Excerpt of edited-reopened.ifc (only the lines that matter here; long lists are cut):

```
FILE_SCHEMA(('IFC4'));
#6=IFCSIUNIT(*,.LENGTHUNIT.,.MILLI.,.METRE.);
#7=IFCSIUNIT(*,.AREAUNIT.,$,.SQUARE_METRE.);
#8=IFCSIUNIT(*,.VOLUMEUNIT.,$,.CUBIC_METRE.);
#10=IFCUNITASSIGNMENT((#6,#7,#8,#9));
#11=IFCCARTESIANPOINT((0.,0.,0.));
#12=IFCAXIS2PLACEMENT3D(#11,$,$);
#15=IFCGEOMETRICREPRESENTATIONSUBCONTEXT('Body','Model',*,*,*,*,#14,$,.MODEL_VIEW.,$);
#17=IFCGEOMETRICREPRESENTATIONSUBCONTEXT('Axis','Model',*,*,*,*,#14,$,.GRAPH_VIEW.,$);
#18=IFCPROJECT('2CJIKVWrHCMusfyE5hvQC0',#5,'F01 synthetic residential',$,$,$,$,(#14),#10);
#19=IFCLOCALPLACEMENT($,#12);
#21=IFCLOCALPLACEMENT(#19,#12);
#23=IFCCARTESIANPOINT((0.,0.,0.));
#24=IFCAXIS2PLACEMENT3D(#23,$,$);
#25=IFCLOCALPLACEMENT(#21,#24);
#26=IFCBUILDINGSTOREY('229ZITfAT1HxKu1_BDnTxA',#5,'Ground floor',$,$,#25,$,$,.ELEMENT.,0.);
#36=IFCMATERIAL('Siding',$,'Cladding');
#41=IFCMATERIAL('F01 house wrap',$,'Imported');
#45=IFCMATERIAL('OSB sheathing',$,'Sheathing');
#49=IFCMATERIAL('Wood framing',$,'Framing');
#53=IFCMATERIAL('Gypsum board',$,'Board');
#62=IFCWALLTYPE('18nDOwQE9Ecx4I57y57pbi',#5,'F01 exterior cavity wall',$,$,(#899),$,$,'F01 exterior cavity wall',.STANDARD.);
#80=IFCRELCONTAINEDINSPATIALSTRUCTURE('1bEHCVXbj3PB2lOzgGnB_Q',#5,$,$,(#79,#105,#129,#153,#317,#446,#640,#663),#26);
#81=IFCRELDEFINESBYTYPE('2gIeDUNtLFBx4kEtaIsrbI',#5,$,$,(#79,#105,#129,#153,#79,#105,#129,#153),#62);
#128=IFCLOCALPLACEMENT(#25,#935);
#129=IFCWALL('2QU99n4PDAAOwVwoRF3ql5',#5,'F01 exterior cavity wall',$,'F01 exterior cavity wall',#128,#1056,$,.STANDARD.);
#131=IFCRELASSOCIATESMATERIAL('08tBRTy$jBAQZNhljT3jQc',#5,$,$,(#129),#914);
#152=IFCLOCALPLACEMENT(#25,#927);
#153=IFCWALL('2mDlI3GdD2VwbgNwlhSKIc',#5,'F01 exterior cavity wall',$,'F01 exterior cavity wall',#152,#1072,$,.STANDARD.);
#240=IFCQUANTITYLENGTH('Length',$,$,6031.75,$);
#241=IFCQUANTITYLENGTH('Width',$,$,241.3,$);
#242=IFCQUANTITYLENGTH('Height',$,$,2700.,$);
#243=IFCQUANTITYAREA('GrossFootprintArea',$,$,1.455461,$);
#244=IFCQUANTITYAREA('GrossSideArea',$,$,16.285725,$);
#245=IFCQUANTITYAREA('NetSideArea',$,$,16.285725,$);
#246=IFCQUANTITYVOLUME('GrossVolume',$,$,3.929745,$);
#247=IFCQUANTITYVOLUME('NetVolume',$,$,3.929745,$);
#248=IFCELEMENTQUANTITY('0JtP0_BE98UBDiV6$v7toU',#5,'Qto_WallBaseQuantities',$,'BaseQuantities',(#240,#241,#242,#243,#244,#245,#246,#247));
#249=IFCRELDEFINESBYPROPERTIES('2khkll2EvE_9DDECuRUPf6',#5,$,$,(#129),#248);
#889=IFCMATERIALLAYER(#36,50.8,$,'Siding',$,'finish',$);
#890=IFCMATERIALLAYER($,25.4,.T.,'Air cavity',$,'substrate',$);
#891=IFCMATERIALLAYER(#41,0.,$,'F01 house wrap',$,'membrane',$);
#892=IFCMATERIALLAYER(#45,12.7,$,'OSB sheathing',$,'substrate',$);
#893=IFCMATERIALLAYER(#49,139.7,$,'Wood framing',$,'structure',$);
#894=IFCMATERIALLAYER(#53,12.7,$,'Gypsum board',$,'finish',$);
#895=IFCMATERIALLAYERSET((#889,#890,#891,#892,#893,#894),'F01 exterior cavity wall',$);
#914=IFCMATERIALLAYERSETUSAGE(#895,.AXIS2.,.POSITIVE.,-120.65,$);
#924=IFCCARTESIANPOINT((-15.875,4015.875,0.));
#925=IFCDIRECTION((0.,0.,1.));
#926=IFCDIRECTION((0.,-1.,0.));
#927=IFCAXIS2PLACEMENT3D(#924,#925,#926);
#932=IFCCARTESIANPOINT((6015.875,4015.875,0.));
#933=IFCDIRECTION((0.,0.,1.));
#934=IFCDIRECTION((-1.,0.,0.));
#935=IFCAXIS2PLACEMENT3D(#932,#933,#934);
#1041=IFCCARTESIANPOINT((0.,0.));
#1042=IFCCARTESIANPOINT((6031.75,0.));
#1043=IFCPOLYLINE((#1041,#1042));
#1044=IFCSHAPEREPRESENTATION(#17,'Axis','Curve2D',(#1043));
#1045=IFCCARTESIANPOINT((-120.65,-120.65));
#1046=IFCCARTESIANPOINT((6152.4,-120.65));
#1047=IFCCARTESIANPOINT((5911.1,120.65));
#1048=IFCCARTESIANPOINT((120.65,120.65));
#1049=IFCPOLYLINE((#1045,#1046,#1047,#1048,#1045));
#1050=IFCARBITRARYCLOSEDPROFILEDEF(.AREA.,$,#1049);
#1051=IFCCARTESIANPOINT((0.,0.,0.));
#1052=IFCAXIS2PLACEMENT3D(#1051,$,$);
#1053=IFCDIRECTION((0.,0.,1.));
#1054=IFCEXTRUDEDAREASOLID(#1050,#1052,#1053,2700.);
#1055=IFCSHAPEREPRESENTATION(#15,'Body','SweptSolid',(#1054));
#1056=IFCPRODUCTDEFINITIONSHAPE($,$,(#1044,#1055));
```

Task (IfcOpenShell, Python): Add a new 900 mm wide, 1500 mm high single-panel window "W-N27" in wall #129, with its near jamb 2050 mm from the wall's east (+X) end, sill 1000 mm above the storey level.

```python
import numpy as np
import ifcopenshell
import ifcopenshell.api.feature
import ifcopenshell.api.geometry
import ifcopenshell.api.pset
import ifcopenshell.api.root
import ifcopenshell.api.spatial
import ifcopenshell.geom
import ifcopenshell.util.element
import ifcopenshell.util.placement
import ifcopenshell.util.representation
import ifcopenshell.util.shape
import ifcopenshell.util.unit

model = ifcopenshell.open("edited-reopened.ifc")
unit_scale = ifcopenshell.util.unit.calculate_unit_scale(model)
area_scale = ifcopenshell.util.unit.calculate_unit_scale(model, "AREAUNIT")
volume_scale = ifcopenshell.util.unit.calculate_unit_scale(model, "VOLUMEUNIT")
settings = ifcopenshell.geom.settings()


def volume(element):
    """Net volume in cubic metres, openings subtracted."""
    shape = ifcopenshell.geom.create_shape(settings, element)
    return ifcopenshell.util.shape.get_volume(shape.geometry)


wall = model.by_guid("2QU99n4PDAAOwVwoRF3ql5")
storey = ifcopenshell.util.element.get_container(wall, ifc_class="IfcBuildingStorey")
context = ifcopenshell.util.representation.get_context(model, "Model", "Body", "MODEL_VIEW")
before = volume(wall)

width, height, from_end, sill = 0.9, 1.5, 2.05, 1  # metres

# The wall runs along its own X axis, and the end named is its -X end.
wall_shape = ifcopenshell.geom.create_shape(settings, wall)
x, y, z = ifcopenshell.util.shape.get_vertices(wall_shape.geometry).T
start = x.min() + from_end
face, thickness = float(y.min()), float(y.max() - y.min())
wall_matrix = ifcopenshell.util.placement.get_local_placement(wall.ObjectPlacement)
level = ifcopenshell.util.placement.get_local_placement(storey.ObjectPlacement)[2, 3]


def in_wall(x, y):
    """Placement at x, y metres in the wall's axes, at sill height."""
    matrix = wall_matrix.copy()
    matrix[:, 3] = wall_matrix @ np.array([x / unit_scale, y / unit_scale, 0.0, 1.0])
    matrix[2, 3] = level + sill / unit_scale
    return matrix


# Opening: a box that overshoots both wall faces by 50 mm.
opening = ifcopenshell.api.root.create_entity(model, ifc_class="IfcOpeningElement", predefined_type="OPENING")
box = ifcopenshell.api.geometry.add_wall_representation(
    model, context=context, length=width, height=height, thickness=thickness + 0.1
)
ifcopenshell.api.geometry.assign_representation(model, product=opening, representation=box)
ifcopenshell.api.geometry.edit_object_placement(model, product=opening, matrix=in_wall(start, face - 0.05), is_si=False)
ifcopenshell.api.feature.add_feature(model, feature=opening, element=wall)

window = ifcopenshell.api.root.create_entity(model, ifc_class="IfcWindow", name="W-N27", predefined_type="WINDOW")
window.OverallWidth, window.OverallHeight = width / unit_scale, height / unit_scale
window.PartitioningType = "SINGLE_PANEL"
body = ifcopenshell.api.geometry.add_window_representation(
    model,
    context=context,
    overall_width=window.OverallWidth,
    overall_height=window.OverallHeight,
    partition_type="SINGLE_PANEL",
)
ifcopenshell.api.geometry.assign_representation(model, product=window, representation=body)
ifcopenshell.api.spatial.assign_container(model, products=[window], relating_structure=storey)
ifcopenshell.api.feature.add_filling(model, opening=opening, element=window)

# Centre the window in the wall's thickness.
ifcopenshell.api.geometry.edit_object_placement(model, product=window, matrix=in_wall(start, face), is_si=False)
window_shape = ifcopenshell.geom.create_shape(settings, window)
depth = ifcopenshell.util.shape.get_vertices(window_shape.geometry)[:, 1]
offset = face + thickness / 2 - (depth.min() + depth.max()) / 2
ifcopenshell.api.geometry.edit_object_placement(model, product=window, matrix=in_wall(start, offset), is_si=False)

after = volume(wall)

# Update the wall's stored quantities.
qto = model.by_id(ifcopenshell.util.element.get_pset(wall, "Qto_WallBaseQuantities", should_inherit=False)["id"])
ifcopenshell.api.pset.edit_qto(model, qto=qto, properties={
    "NetSideArea": after / thickness / area_scale,
    "NetVolume": after / volume_scale,
})

print(f"wall volume {before:.3f} -> {after:.3f} m3")

model.write("edited-reopened_rev.ifc")
```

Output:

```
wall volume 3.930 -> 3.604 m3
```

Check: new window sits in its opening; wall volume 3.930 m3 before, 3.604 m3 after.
